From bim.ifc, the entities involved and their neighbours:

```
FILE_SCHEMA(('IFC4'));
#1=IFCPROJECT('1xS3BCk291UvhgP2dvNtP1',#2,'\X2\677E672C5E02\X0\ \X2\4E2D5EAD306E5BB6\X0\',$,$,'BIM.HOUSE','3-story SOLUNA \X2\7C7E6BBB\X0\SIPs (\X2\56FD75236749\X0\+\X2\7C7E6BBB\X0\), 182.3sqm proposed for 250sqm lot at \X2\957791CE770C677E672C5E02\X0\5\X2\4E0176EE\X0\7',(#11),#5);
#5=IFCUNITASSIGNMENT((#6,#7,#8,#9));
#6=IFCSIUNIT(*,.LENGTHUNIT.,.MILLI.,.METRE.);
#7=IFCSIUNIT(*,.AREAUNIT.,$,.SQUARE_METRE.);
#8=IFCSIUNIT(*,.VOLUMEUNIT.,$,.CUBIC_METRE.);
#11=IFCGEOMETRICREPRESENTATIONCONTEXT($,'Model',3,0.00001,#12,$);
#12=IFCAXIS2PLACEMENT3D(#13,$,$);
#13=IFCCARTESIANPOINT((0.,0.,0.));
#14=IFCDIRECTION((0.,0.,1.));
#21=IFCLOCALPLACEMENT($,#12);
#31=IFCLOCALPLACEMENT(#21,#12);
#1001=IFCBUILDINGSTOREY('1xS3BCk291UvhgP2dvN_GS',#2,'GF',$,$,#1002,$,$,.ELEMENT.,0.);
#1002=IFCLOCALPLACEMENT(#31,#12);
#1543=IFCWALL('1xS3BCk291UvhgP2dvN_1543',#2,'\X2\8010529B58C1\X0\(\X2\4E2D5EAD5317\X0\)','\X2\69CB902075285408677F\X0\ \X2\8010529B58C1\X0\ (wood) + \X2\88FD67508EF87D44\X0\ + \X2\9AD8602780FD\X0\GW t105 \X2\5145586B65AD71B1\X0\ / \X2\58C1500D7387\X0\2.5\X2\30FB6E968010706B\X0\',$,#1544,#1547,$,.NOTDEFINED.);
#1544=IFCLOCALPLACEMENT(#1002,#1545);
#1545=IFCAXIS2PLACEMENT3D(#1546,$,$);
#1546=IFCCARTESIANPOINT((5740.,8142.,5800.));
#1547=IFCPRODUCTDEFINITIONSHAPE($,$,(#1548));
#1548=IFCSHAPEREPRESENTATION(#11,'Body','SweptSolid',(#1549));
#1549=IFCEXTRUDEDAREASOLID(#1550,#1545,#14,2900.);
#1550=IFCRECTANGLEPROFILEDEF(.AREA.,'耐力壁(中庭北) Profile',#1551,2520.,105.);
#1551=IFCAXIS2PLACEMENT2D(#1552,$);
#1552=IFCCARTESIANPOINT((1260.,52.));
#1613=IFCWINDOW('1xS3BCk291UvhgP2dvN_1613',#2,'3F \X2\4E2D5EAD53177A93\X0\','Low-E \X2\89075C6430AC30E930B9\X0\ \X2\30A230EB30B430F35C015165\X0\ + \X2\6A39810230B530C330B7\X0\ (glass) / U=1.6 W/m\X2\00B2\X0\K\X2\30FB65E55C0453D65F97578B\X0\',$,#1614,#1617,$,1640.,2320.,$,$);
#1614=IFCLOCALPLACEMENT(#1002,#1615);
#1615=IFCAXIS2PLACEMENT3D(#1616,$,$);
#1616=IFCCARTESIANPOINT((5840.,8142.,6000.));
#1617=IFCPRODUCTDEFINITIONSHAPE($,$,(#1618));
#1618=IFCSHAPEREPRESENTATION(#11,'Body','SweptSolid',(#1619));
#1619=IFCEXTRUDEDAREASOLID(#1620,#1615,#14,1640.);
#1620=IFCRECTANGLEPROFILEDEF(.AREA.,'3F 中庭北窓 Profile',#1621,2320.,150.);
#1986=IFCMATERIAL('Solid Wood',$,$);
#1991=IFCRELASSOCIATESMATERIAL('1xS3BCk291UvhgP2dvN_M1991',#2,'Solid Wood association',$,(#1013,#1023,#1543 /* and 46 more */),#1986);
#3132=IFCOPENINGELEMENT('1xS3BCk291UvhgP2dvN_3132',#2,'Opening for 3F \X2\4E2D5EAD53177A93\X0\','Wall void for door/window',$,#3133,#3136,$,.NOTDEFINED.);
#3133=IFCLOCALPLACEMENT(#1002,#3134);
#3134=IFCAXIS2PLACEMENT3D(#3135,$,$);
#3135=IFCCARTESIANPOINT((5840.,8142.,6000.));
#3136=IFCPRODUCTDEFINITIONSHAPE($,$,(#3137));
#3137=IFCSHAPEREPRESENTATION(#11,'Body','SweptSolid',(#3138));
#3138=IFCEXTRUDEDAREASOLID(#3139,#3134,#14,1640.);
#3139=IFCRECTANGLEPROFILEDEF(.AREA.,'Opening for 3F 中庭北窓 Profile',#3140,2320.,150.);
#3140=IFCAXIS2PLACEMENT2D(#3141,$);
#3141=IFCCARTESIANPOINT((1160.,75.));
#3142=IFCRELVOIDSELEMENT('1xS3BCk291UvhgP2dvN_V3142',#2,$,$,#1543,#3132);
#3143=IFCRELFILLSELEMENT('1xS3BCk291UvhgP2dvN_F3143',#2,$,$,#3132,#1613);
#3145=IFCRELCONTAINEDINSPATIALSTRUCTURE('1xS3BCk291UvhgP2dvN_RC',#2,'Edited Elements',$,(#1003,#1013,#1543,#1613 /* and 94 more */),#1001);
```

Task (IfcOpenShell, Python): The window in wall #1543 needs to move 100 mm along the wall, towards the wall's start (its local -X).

```python
import ifcopenshell
import ifcopenshell.api.geometry
import ifcopenshell.util.placement

model = ifcopenshell.open("bim.ifc")

window = model.by_id(1613)
opening = window.FillsVoids[0].RelatingOpeningElement
wall = opening.VoidsElements[0].RelatingBuildingElement

wall_matrix = ifcopenshell.util.placement.get_local_placement(wall.ObjectPlacement)
shift = wall_matrix[:3, 0] * -100.0
before = ifcopenshell.util.placement.get_local_placement(window.ObjectPlacement)[:3, 3].copy()

# The window is not placed relative to its opening, so move both.
for product in (opening, window):
    matrix = ifcopenshell.util.placement.get_local_placement(product.ObjectPlacement)
    matrix[:3, 3] += shift
    ifcopenshell.api.geometry.edit_object_placement(model, product=product, matrix=matrix, is_si=False)

after = ifcopenshell.util.placement.get_local_placement(window.ObjectPlacement)[:3, 3]
print("window moved by", (after - before).round(3) + 0.0)

model.write("bim_edited.ifc")
```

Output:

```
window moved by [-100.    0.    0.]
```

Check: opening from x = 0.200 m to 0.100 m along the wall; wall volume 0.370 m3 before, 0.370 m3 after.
